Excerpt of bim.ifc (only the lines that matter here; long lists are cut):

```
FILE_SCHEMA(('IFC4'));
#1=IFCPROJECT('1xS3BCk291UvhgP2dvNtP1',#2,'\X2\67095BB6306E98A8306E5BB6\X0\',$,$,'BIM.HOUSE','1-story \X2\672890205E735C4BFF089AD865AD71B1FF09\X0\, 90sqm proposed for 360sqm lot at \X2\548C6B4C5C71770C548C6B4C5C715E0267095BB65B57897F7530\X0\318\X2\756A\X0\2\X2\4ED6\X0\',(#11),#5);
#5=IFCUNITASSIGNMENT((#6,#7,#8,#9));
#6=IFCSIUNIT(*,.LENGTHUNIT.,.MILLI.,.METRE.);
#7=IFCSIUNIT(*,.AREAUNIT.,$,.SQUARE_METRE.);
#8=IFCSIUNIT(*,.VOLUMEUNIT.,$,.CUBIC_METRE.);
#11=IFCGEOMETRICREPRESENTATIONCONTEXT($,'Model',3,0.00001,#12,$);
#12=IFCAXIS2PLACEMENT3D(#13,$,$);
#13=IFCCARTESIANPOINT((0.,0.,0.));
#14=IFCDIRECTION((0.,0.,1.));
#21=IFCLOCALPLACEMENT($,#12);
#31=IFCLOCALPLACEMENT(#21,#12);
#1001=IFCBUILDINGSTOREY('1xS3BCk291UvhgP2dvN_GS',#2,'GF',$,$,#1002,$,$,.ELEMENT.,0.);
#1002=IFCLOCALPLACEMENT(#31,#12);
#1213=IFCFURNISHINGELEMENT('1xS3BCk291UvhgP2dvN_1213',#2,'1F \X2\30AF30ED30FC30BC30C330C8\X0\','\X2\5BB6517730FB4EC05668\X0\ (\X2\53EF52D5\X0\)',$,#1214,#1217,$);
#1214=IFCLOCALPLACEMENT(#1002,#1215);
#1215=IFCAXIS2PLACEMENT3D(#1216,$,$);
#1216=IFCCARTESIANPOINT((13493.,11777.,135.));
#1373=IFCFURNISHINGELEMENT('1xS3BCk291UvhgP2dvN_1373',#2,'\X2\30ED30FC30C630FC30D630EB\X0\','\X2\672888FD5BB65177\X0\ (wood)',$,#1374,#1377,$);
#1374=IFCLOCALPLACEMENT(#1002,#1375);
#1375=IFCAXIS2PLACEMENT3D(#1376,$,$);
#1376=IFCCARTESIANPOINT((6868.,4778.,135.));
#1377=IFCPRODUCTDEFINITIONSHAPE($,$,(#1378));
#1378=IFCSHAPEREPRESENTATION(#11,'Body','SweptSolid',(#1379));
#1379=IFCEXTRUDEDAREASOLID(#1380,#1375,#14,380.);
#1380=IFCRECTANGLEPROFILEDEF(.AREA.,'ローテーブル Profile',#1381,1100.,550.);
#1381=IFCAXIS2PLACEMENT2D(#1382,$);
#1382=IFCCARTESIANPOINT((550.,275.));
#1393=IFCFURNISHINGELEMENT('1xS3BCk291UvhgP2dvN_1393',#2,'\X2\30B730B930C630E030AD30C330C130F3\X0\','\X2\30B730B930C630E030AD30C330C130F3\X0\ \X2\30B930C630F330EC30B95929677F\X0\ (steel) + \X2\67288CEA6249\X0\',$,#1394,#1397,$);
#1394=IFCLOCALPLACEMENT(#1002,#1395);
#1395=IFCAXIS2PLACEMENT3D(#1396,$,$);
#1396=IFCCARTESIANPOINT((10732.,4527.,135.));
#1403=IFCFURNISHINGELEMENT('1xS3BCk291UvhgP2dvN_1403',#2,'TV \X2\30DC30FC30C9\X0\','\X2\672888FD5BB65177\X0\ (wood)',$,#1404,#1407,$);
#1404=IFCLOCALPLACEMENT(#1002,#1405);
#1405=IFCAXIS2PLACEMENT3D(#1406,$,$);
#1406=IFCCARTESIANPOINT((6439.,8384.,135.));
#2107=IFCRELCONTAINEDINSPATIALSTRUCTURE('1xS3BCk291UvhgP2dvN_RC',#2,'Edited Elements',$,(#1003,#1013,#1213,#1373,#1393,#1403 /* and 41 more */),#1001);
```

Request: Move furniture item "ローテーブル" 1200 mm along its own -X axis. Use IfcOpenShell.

```python
import ifcopenshell
import ifcopenshell.api.geometry
import ifcopenshell.util.placement
import ifcopenshell.util.unit

model = ifcopenshell.open("bim.ifc")
unit_scale = ifcopenshell.util.unit.calculate_unit_scale(model)

item = model.by_id(1373)
matrix = ifcopenshell.util.placement.get_local_placement(item.ObjectPlacement)
matrix[:3, 3] -= matrix[:3, 0] * 1.2 / unit_scale
ifcopenshell.api.geometry.edit_object_placement(model, product=item, matrix=matrix, is_si=False)

print(ifcopenshell.util.placement.get_local_placement(item.ObjectPlacement).round(3) + 0.0)

model.write("bim_rev.ifc")
```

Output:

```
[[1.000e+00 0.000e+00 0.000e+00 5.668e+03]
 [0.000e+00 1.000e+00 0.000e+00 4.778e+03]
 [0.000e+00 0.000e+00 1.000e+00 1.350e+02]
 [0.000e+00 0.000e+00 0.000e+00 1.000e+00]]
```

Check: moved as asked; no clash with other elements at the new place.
